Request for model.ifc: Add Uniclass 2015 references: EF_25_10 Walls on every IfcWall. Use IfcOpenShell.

First a look at what the model holds.

```python
import ifcopenshell

model = ifcopenshell.open("model.ifc")
print(model.schema)
print("classifications:", [c.Name for c in model.by_type("IfcClassification")])
for ifc_class in ("IfcDoor", "IfcRoof", "IfcStair", "IfcWall", "IfcWindow"):
    print(ifc_class, len(model.by_type(ifc_class)))
```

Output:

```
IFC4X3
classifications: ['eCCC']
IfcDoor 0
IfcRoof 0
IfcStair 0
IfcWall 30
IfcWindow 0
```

```python
import ifcopenshell
import ifcopenshell.api.classification

model = ifcopenshell.open("model.ifc")

system = ifcopenshell.api.classification.add_classification(model, classification="Uniclass 2015")

codes = {
    "IfcWall": ("EF_25_10", "Walls"),
}
for ifc_class, (code, name) in codes.items():
    products = model.by_type(ifc_class)
    ifcopenshell.api.classification.add_reference(
        model, products=products, classification=system, identification=code, name=name
    )
    print(code, len(products))

model.write("model-out.ifc")
```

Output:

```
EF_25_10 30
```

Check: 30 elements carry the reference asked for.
